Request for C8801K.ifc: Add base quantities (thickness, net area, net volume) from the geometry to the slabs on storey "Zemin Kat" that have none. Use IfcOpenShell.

First a look at what the model holds.

```python
import ifcopenshell
import ifcopenshell.util.element
import ifcopenshell.util.unit

model = ifcopenshell.open("C8801K.ifc")
print(model.schema)
for unit_type in ("LENGTHUNIT", "AREAUNIT", "VOLUMEUNIT"):
    print(unit_type, ifcopenshell.util.unit.calculate_unit_scale(model, unit_type))
storey = next(s for s in model.by_type("IfcBuildingStorey") if s.Name == "Zemin Kat")
slabs = [e for e in ifcopenshell.util.element.get_decomposition(storey) if e.is_a("IfcSlab")]
for e in sorted(slabs, key=lambda e: e.id()):
    print(e.id(), e.is_a(), e.Name, list(ifcopenshell.util.element.get_psets(e, qtos_only=True)), sep=" | ")
```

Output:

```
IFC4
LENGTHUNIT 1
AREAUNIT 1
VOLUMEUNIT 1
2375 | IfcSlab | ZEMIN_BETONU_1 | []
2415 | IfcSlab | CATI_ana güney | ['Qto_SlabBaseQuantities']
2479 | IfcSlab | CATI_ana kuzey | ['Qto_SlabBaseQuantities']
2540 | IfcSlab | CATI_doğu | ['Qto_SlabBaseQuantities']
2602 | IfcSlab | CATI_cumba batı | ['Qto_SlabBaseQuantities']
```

```python
import ifcopenshell
import ifcopenshell.api.pset
import ifcopenshell.geom
import ifcopenshell.util.element
import ifcopenshell.util.shape
import ifcopenshell.util.unit

model = ifcopenshell.open("C8801K.ifc")
unit_scale = ifcopenshell.util.unit.calculate_unit_scale(model)
area_scale = ifcopenshell.util.unit.calculate_unit_scale(model, "AREAUNIT")
volume_scale = ifcopenshell.util.unit.calculate_unit_scale(model, "VOLUMEUNIT")
settings = ifcopenshell.geom.settings()

storey = next(s for s in model.by_type("IfcBuildingStorey") if s.Name == "Zemin Kat")
slabs = [e for e in ifcopenshell.util.element.get_decomposition(storey) if e.is_a("IfcSlab")]

for e in sorted(slabs, key=lambda e: e.id()):
    if ifcopenshell.util.element.get_psets(e, qtos_only=True, should_inherit=False):
        continue
    # Geometry comes back in metres, in the element's own axes.
    shape = ifcopenshell.geom.create_shape(settings, e)
    values = {
        "Width": ifcopenshell.util.shape.get_z(shape.geometry) / unit_scale,
        "NetArea": ifcopenshell.util.shape.get_footprint_area(shape.geometry) / area_scale,
        "NetVolume": ifcopenshell.util.shape.get_volume(shape.geometry) / volume_scale,
    }
    qto = ifcopenshell.api.pset.add_qto(model, product=e, name="Qto_SlabBaseQuantities")
    ifcopenshell.api.pset.edit_qto(model, qto=qto, properties=values)
    print(e.id(), {k: round(v, 3) for k, v in values.items()})

model.write("C8801K_rev.ifc")
```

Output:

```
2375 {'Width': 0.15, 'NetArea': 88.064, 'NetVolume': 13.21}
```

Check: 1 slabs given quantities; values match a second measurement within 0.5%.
